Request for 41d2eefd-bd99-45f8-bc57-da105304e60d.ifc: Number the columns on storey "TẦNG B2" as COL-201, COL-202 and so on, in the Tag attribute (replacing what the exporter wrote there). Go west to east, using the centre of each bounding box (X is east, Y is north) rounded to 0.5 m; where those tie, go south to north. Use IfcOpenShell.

First a look at what the model holds.

```python
import ifcopenshell
import ifcopenshell.util.element
import ifcopenshell.util.placement

model = ifcopenshell.open("41d2eefd-bd99-45f8-bc57-da105304e60d.ifc")
print(model.schema)
storey = next(s for s in model.by_type("IfcBuildingStorey") if s.Name == "TẦNG B2")
columns = [e for e in ifcopenshell.util.element.get_decomposition(storey) if e.is_a("IfcColumn")]
for e in sorted(columns, key=lambda e: e.id()):
    origin = ifcopenshell.util.placement.get_local_placement(e.ObjectPlacement)[:3, 3]
    print(e.id(), e.Tag, e.Name, origin.round(2) + 0.0, sep=" | ")
```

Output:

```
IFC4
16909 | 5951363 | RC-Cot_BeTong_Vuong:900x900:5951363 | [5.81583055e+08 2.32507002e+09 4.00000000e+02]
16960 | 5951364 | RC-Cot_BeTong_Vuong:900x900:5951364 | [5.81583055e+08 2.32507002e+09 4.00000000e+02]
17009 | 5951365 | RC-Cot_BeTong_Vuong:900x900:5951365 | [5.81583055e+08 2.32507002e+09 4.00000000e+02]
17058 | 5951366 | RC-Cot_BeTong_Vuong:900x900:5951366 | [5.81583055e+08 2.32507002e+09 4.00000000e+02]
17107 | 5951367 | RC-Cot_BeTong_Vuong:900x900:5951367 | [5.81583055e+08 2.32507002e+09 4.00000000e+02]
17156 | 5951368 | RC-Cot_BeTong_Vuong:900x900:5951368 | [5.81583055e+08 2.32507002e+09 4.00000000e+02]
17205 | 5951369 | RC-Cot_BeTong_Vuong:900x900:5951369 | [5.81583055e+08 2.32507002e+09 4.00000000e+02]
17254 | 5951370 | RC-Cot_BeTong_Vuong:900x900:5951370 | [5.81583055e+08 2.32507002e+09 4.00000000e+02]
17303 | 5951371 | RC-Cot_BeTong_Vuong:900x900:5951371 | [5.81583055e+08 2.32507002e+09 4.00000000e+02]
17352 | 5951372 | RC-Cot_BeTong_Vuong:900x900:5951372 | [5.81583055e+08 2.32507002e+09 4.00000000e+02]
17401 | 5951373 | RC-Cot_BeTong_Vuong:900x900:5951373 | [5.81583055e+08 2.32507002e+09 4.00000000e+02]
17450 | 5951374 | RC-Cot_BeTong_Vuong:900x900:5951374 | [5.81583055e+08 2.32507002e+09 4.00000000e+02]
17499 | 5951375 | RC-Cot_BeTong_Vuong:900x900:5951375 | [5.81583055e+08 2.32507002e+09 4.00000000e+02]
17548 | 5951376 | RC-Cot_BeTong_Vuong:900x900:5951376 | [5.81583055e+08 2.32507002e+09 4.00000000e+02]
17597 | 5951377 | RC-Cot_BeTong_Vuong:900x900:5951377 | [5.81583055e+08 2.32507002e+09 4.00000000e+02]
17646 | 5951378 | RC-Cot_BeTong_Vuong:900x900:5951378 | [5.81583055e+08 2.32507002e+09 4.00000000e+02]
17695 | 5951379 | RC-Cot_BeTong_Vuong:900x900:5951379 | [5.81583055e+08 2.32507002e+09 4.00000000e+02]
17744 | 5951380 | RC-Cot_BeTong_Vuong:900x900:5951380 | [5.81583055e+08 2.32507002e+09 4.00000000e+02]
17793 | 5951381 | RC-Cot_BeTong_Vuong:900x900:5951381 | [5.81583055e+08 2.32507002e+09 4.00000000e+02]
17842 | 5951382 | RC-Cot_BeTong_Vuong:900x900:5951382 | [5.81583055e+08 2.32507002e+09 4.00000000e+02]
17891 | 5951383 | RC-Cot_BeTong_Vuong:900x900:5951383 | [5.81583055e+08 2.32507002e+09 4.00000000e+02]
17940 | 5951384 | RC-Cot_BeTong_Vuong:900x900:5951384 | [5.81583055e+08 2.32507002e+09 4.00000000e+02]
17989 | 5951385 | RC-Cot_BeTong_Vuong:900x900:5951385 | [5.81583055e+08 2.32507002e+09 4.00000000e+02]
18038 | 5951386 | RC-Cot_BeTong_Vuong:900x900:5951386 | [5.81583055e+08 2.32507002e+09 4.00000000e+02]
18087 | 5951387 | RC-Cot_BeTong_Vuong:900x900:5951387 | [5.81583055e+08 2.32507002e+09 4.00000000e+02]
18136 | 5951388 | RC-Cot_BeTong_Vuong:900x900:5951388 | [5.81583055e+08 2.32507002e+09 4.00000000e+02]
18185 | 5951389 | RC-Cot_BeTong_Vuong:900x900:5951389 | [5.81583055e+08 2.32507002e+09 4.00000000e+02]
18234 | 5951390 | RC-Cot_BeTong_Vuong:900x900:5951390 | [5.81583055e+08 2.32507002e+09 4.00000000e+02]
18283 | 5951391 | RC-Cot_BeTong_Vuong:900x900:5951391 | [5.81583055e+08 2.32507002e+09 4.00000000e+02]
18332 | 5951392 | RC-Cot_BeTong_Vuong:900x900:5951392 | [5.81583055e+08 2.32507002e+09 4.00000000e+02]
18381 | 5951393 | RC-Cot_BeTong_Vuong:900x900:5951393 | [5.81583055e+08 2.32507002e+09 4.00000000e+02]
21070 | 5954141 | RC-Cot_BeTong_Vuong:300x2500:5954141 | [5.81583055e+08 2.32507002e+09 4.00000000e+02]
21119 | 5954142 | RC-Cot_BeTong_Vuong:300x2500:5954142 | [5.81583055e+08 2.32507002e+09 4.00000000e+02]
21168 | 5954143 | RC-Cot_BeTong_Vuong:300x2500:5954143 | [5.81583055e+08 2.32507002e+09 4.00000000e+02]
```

```python
import ifcopenshell
import ifcopenshell.geom
import ifcopenshell.util.element
import ifcopenshell.util.shape

model = ifcopenshell.open("41d2eefd-bd99-45f8-bc57-da105304e60d.ifc")
settings = ifcopenshell.geom.settings()
settings.set("use-world-coords", True)


def centre(element):
    shape = ifcopenshell.geom.create_shape(settings, element)
    return ifcopenshell.util.shape.get_bbox_centroid(shape.geometry)


storey = next(s for s in model.by_type("IfcBuildingStorey") if s.Name == "TẦNG B2")
columns = [e for e in ifcopenshell.util.element.get_decomposition(storey) if e.is_a("IfcColumn")]

# Insertion points can sit at a corner or the storey origin, so sort by the geometry (in metres).
centres = {e: centre(e) for e in columns}
columns.sort(key=lambda e: (round(centres[e][0] / 0.5), centres[e][1]))

for i, e in enumerate(columns, start=1):
    number = f"COL-2{i:02d}"
    e.Tag = number
    print(e.id(), number)

model.write("41d2eefd-bd99-45f8-bc57-da105304e60d_v2.ifc")
```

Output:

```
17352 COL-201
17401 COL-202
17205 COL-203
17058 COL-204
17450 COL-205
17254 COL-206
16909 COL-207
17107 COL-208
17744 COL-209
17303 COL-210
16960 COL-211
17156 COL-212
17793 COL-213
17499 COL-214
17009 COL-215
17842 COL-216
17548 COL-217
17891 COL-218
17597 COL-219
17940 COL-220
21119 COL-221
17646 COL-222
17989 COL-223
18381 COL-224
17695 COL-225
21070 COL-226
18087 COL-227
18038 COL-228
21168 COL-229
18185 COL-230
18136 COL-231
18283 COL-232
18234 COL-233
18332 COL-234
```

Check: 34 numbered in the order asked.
